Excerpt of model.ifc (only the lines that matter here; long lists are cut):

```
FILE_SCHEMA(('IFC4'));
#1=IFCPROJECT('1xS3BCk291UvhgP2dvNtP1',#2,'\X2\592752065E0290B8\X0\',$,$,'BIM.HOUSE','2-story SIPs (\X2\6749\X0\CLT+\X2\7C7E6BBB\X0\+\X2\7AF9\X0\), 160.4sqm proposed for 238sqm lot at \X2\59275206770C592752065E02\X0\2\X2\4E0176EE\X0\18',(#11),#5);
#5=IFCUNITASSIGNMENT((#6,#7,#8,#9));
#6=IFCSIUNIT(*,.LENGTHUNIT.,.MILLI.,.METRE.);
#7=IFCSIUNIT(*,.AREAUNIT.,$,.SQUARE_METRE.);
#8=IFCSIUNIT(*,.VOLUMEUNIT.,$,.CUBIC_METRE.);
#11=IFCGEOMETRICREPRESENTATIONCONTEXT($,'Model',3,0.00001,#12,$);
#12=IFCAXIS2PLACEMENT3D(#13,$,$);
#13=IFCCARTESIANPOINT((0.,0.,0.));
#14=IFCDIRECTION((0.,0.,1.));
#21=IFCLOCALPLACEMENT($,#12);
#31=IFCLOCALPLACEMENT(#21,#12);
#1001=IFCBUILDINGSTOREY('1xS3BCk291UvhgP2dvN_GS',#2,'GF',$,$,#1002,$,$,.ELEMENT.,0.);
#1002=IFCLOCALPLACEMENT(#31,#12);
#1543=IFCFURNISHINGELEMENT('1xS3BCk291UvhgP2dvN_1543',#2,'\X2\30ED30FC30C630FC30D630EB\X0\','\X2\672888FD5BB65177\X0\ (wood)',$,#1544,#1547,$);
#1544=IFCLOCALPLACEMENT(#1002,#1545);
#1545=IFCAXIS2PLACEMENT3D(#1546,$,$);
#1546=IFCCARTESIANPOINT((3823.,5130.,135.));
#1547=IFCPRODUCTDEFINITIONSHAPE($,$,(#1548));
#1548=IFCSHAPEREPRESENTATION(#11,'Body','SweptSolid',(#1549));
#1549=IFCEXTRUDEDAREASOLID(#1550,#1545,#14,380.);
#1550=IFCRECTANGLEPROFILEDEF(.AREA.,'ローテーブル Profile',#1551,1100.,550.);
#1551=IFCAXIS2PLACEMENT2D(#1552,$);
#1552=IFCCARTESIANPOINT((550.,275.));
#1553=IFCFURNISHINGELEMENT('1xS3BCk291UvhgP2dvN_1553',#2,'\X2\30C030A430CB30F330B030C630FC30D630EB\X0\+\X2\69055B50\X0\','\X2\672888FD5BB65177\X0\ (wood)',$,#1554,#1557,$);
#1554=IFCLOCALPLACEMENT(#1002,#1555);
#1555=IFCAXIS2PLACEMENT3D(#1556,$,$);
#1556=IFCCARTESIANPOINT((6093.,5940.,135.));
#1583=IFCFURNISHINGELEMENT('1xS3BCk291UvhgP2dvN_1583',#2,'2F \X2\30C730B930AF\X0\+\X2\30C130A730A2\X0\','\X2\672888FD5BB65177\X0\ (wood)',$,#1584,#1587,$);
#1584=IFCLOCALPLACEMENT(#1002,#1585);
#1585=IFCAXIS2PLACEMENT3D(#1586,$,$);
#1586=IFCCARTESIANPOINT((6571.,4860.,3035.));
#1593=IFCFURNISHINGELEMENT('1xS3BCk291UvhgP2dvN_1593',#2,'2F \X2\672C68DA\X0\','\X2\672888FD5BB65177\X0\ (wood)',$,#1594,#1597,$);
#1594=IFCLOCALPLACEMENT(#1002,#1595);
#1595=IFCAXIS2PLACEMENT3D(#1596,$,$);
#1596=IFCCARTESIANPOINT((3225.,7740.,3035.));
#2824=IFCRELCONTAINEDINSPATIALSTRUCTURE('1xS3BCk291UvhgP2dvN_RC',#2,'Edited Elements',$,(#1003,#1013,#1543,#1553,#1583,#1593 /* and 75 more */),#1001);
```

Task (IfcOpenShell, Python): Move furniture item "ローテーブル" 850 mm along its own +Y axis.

```python
import ifcopenshell
import ifcopenshell.api.geometry
import ifcopenshell.util.placement
import ifcopenshell.util.unit

model = ifcopenshell.open("model.ifc")
unit_scale = ifcopenshell.util.unit.calculate_unit_scale(model)

item = model.by_id(1543)
matrix = ifcopenshell.util.placement.get_local_placement(item.ObjectPlacement)
matrix[:3, 3] += matrix[:3, 1] * 0.85 / unit_scale
ifcopenshell.api.geometry.edit_object_placement(model, product=item, matrix=matrix, is_si=False)

print(ifcopenshell.util.placement.get_local_placement(item.ObjectPlacement).round(3) + 0.0)

model.write("model-out.ifc")
```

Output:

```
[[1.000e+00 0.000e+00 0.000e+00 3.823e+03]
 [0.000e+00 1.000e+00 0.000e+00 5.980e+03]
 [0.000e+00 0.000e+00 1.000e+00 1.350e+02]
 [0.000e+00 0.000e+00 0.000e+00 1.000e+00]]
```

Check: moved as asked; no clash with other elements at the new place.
